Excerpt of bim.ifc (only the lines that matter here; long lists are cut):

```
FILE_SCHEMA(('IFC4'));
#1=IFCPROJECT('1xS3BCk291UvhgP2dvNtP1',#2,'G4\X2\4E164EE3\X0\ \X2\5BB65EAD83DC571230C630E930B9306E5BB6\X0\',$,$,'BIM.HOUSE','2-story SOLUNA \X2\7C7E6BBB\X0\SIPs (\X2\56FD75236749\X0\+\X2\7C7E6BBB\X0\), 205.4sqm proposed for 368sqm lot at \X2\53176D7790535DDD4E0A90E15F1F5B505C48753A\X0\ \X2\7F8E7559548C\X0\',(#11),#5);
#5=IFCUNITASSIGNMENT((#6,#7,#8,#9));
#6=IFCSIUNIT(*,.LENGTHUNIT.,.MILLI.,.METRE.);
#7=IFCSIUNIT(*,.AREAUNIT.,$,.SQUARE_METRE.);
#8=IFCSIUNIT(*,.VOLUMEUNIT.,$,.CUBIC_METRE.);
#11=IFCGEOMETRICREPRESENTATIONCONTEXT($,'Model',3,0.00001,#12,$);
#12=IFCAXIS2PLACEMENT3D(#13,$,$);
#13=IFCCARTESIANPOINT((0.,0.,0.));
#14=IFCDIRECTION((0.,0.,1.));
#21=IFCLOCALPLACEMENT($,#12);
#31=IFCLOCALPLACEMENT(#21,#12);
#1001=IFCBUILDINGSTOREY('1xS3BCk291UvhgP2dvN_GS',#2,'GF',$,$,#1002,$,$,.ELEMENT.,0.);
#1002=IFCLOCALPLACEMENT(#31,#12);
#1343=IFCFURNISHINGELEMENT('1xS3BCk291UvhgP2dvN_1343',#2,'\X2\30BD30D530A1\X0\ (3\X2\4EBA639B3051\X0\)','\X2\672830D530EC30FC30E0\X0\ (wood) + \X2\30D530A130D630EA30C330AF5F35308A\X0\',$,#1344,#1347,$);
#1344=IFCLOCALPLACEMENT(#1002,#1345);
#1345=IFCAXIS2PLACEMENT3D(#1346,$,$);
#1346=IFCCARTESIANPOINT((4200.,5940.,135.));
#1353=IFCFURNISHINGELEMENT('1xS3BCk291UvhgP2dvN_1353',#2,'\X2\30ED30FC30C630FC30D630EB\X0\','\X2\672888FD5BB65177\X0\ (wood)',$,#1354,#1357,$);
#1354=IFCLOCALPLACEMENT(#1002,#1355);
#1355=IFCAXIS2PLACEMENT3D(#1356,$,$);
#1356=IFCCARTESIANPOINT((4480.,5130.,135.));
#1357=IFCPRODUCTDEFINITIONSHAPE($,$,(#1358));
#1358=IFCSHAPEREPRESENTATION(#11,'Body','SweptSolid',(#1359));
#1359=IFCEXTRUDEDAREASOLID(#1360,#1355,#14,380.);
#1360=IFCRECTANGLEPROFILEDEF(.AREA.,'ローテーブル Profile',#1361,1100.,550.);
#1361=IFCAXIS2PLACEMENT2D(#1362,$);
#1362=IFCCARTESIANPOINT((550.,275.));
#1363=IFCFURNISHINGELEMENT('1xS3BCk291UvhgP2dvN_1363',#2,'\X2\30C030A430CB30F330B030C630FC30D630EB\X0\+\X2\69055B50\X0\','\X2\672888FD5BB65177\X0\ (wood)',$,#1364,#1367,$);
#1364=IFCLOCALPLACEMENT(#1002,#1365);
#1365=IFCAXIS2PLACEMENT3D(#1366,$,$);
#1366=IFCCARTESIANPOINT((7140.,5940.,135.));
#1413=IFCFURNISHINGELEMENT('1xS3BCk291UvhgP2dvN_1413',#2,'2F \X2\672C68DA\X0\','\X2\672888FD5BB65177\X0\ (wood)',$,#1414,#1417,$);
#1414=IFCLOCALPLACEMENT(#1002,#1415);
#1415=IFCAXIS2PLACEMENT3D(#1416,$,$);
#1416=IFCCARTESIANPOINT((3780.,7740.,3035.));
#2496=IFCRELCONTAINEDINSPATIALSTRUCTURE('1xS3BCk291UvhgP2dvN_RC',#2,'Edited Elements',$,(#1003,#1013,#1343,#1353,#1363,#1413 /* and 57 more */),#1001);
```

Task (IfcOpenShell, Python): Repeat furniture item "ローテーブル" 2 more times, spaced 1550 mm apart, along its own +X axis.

```python
import ifcopenshell
import ifcopenshell.api.geometry
import ifcopenshell.api.root
import ifcopenshell.util.element
import ifcopenshell.util.placement

model = ifcopenshell.open("bim.ifc")


def reuse_history(source, copy):
    """copy_class also copies each property set's owner history, people and application; keep the originals."""
    for rel in copy.IsDefinedBy:
        if rel.is_a("IfcRelDefinesByProperties") and (history := rel.RelatingPropertyDefinition.OwnerHistory):
            rel.RelatingPropertyDefinition.OwnerHistory = source.OwnerHistory
            ifcopenshell.util.element.remove_deep2(model, history)


source = model.by_guid("1xS3BCk291UvhgP2dvN_1353")
base = ifcopenshell.util.placement.get_local_placement(source.ObjectPlacement)
step = base[:3, 0] * 1550.0

for i in range(1, 3):
    copy = ifcopenshell.api.root.copy_class(model, product=source)
    copy.Representation = ifcopenshell.util.element.copy_deep(
        model, source.Representation, exclude=["IfcGeometricRepresentationContext", "IfcRepresentationMap"]
    )
    reuse_history(source, copy)
    matrix = base.copy()
    matrix[:3, 3] += i * step
    print("added at", matrix[:3, 3].round(3) + 0.0)
    ifcopenshell.api.geometry.edit_object_placement(model, product=copy, matrix=matrix, is_si=False)

model.write("bim_v2.ifc")
```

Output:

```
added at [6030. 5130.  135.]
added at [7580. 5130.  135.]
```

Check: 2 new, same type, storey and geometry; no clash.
